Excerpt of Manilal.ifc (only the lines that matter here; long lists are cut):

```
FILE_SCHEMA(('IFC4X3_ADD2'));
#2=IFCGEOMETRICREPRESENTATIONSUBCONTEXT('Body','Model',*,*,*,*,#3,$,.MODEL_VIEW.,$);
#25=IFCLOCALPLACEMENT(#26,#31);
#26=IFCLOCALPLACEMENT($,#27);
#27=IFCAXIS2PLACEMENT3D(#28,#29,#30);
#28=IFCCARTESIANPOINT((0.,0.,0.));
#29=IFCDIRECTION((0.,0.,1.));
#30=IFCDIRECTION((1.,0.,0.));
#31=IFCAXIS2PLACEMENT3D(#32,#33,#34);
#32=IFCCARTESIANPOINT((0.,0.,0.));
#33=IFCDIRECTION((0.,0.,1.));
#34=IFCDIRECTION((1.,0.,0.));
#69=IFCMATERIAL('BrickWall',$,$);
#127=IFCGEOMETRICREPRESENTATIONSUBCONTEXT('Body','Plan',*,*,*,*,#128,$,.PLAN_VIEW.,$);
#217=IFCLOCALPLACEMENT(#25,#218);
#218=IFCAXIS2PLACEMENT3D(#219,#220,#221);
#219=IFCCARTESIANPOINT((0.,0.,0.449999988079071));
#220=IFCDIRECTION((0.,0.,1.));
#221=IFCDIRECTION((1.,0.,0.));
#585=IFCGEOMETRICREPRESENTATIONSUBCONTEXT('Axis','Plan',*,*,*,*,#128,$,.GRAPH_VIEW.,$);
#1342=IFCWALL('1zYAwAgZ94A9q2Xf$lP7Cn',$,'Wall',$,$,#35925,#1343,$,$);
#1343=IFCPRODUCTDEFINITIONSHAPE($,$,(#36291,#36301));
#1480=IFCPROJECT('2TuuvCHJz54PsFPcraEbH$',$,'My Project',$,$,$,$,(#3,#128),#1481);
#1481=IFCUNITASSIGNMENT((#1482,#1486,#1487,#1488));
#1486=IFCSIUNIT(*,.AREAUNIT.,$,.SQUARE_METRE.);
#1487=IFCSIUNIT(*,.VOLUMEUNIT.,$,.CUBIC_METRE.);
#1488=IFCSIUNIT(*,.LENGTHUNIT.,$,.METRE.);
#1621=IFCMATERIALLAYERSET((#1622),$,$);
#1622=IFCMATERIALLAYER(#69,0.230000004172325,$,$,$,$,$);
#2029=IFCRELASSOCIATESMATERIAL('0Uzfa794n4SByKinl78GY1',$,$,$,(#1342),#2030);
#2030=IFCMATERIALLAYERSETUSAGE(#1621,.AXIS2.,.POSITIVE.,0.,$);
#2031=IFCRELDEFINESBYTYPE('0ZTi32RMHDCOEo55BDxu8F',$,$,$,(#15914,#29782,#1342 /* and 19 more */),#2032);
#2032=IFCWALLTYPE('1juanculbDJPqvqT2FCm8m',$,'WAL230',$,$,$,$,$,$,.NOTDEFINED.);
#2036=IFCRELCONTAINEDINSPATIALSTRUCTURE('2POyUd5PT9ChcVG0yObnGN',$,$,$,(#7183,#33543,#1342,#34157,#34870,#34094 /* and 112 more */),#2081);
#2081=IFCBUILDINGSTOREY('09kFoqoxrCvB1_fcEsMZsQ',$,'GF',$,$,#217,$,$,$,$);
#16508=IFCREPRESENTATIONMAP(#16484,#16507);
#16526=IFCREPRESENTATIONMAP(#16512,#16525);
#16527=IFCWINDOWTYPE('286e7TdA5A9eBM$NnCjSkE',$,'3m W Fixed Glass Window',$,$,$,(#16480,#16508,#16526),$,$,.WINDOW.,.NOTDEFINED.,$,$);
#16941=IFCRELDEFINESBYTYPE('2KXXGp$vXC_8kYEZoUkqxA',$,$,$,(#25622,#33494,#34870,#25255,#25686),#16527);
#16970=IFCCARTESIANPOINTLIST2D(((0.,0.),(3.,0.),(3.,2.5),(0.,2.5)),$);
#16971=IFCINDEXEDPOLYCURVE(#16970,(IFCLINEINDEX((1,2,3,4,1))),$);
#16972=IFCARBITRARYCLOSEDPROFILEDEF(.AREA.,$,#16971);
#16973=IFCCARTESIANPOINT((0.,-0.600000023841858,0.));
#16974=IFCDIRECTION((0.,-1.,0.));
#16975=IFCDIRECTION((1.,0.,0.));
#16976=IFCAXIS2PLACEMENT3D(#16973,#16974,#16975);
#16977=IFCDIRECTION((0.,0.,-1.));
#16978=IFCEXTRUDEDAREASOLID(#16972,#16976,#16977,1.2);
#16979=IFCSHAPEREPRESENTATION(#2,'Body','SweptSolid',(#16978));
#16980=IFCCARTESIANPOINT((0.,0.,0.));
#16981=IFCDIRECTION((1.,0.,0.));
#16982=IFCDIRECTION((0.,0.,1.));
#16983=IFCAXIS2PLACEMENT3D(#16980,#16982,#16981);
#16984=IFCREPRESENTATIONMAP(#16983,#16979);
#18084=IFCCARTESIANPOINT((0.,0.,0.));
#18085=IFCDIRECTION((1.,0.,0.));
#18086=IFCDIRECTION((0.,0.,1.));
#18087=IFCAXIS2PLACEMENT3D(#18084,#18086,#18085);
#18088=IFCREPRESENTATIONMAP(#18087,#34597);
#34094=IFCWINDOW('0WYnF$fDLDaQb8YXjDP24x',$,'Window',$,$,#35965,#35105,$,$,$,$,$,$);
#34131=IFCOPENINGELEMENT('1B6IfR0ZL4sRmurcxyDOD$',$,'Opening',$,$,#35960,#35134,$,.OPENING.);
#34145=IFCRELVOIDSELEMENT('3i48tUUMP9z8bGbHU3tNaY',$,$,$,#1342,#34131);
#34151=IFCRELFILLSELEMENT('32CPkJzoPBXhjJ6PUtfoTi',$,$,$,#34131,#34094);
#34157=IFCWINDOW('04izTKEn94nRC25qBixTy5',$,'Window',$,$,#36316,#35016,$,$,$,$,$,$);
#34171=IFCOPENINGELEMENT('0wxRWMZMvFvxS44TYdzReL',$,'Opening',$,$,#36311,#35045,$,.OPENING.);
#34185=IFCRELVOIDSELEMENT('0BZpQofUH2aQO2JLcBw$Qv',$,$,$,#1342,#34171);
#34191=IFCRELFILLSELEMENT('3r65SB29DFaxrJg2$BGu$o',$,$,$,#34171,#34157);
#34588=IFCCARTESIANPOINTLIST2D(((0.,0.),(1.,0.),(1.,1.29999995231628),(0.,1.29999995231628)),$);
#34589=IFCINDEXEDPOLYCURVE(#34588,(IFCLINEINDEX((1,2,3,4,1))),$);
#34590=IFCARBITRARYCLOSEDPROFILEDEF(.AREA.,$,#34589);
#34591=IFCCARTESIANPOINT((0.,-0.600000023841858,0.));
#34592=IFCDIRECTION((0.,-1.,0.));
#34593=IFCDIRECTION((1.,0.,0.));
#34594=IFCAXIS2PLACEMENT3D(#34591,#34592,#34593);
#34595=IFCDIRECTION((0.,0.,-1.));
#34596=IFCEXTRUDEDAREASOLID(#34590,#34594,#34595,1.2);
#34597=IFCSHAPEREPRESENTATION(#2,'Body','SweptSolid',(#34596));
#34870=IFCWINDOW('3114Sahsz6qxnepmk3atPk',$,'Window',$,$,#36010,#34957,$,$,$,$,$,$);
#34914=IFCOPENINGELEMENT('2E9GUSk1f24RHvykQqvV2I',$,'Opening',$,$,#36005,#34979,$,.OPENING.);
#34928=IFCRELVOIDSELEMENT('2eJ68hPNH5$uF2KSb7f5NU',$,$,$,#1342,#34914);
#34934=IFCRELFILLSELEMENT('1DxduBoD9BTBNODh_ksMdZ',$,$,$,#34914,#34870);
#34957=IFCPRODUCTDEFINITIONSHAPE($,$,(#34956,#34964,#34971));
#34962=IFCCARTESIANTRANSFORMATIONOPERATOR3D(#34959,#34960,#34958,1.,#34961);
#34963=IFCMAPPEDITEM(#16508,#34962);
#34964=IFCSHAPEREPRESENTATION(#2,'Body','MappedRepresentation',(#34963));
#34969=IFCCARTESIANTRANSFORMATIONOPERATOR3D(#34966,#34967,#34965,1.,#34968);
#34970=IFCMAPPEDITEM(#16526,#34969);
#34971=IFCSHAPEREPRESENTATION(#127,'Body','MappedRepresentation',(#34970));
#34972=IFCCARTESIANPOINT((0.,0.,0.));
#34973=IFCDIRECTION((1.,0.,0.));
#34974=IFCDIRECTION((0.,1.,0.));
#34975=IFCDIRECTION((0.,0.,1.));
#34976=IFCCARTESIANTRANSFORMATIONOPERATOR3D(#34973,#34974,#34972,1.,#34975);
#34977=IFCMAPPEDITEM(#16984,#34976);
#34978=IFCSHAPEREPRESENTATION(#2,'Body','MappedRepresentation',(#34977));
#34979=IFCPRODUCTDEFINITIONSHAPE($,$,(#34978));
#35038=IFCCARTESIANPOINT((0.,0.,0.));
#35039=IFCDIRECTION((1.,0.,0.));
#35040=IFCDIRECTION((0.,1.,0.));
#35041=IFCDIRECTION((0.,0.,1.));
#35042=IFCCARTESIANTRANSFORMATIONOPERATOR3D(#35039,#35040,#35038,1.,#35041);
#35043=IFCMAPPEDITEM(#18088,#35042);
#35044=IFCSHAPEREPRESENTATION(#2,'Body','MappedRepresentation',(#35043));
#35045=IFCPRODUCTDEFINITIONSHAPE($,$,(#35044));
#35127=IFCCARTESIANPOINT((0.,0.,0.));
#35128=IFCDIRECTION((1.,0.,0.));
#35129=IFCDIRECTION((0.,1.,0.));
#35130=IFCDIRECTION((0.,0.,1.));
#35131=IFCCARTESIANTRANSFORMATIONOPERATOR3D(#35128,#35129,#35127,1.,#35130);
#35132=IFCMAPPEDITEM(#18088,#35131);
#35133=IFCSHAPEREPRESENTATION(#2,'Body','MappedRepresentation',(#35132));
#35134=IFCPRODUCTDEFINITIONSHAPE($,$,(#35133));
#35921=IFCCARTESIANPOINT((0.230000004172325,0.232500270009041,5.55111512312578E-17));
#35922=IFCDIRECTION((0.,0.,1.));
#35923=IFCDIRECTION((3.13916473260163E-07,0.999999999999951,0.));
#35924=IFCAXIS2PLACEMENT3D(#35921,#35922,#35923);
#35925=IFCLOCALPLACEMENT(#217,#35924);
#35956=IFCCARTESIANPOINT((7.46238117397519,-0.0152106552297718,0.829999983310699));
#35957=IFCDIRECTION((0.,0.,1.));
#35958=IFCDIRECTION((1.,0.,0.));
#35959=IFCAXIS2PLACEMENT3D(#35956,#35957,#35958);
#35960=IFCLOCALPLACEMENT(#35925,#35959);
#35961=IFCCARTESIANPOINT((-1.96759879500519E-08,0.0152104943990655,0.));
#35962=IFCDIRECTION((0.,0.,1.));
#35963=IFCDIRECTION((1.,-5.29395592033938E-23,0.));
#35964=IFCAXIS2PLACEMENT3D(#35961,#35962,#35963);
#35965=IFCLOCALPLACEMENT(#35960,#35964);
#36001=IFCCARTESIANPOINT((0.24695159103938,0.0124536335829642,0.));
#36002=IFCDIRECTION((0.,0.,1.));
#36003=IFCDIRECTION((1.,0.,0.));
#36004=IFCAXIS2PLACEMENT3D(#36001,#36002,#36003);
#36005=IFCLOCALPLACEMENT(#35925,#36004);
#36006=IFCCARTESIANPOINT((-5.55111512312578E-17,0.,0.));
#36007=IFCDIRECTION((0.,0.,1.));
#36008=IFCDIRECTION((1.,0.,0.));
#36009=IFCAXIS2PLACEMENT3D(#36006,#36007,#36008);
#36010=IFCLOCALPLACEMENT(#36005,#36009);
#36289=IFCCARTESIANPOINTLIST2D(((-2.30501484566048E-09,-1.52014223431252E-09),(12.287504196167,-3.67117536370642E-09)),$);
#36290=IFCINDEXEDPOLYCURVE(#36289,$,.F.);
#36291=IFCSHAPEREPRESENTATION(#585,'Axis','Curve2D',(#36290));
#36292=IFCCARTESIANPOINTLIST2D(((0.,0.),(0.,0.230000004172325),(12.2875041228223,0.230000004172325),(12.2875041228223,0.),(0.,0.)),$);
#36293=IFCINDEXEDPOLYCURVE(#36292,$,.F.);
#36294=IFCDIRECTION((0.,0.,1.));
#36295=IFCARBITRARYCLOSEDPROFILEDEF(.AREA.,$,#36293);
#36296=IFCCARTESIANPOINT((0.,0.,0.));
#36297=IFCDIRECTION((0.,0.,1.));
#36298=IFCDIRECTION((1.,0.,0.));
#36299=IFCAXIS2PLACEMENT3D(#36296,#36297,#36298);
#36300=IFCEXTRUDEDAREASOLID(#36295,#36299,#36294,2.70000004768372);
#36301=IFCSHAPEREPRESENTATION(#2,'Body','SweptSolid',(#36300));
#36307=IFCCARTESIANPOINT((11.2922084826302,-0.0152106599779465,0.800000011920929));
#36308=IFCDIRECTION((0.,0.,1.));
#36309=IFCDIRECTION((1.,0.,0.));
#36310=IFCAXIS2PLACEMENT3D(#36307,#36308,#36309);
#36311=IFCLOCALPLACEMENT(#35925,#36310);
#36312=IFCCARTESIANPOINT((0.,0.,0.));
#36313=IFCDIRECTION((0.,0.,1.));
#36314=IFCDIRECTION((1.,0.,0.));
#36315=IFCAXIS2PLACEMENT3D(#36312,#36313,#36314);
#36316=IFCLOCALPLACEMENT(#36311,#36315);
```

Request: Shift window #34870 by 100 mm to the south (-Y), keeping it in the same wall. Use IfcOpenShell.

```python
import ifcopenshell
import ifcopenshell.api.geometry
import ifcopenshell.util.placement
import ifcopenshell.util.unit

model = ifcopenshell.open("Manilal.ifc")
unit_scale = ifcopenshell.util.unit.calculate_unit_scale(model)

window = model.by_id(34870)
opening = window.FillsVoids[0].RelatingOpeningElement
wall = opening.VoidsElements[0].RelatingBuildingElement

wall_matrix = ifcopenshell.util.placement.get_local_placement(wall.ObjectPlacement)
shift = wall_matrix[:3, 0] * -0.1 / unit_scale
before = ifcopenshell.util.placement.get_local_placement(window.ObjectPlacement)[:3, 3].copy()

# The window is placed relative to its opening, so it follows when the opening moves.
matrix = ifcopenshell.util.placement.get_local_placement(opening.ObjectPlacement)
matrix[:3, 3] += shift
ifcopenshell.api.geometry.edit_object_placement(
    model, product=opening, matrix=matrix, is_si=False, should_transform_children=True
)

after = ifcopenshell.util.placement.get_local_placement(window.ObjectPlacement)[:3, 3]
print("window moved by", (after - before).round(3) + 0.0)

model.write("Manilal_v2.ifc")
```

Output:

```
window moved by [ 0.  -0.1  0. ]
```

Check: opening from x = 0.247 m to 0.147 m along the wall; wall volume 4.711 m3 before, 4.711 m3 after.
